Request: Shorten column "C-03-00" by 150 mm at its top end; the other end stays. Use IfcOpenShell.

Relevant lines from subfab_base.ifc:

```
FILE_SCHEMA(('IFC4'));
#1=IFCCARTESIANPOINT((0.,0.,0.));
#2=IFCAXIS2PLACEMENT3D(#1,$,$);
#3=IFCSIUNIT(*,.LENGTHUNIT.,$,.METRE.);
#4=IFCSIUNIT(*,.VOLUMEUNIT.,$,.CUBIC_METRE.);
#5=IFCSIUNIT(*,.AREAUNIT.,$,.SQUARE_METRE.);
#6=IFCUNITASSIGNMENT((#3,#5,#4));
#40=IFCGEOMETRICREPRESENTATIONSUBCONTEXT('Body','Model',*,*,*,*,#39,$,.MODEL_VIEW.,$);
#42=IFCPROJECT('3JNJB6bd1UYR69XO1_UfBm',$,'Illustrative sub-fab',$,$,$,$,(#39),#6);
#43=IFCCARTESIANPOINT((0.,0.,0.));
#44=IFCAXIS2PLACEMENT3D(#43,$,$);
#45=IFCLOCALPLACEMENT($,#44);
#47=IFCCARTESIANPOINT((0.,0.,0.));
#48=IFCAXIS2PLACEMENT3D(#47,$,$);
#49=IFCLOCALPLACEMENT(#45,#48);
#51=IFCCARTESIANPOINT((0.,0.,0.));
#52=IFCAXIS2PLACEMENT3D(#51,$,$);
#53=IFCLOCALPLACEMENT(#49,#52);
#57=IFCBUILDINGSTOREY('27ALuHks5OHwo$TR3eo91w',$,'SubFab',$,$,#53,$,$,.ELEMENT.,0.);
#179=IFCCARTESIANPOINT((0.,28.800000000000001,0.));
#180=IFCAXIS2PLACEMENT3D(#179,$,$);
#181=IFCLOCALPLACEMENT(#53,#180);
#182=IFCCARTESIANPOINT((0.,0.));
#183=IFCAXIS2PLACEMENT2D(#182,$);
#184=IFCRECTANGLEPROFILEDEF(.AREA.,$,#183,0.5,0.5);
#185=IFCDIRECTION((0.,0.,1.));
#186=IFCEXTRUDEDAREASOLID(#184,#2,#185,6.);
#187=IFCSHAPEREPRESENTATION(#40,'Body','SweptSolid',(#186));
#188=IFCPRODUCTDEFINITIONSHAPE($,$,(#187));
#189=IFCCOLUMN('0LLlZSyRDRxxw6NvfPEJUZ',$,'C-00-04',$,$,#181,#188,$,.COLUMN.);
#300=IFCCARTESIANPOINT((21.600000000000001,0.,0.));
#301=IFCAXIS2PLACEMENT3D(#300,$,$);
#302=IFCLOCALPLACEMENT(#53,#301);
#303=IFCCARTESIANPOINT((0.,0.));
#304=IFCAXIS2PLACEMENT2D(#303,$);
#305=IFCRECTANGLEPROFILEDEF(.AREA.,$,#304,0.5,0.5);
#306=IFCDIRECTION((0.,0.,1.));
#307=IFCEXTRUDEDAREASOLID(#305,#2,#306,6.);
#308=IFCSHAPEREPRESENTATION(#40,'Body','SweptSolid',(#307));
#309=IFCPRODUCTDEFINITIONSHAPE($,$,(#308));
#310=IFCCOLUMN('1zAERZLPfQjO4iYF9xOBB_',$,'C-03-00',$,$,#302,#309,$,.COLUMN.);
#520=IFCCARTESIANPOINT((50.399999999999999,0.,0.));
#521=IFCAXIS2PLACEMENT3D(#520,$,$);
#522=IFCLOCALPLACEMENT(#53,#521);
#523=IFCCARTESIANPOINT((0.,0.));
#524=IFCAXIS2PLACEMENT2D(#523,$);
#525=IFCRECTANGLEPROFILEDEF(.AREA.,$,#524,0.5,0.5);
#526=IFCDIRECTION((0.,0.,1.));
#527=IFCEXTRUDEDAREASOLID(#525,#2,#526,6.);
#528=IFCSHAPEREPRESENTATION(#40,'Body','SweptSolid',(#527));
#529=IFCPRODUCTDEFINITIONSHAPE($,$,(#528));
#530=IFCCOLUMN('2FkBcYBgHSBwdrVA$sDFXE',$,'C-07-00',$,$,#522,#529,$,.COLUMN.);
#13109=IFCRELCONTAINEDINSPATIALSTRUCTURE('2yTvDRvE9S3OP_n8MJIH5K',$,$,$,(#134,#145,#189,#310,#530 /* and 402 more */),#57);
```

```python
import ifcopenshell
import ifcopenshell.util.representation

model = ifcopenshell.open("subfab_base.ifc")

member = model.by_guid("1zAERZLPfQjO4iYF9xOBB_")
change = -0.15

# The extrusion runs towards the end named, so only its depth changes.
body = ifcopenshell.util.representation.get_representation(member, "Model", "Body")
solid = body.Items[0]
old_length = solid.Depth
solid.Depth += change

print(f"length {old_length:g} -> {solid.Depth:g}")

model.write("subfab_base_rev.ifc")
```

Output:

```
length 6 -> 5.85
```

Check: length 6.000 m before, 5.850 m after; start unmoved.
